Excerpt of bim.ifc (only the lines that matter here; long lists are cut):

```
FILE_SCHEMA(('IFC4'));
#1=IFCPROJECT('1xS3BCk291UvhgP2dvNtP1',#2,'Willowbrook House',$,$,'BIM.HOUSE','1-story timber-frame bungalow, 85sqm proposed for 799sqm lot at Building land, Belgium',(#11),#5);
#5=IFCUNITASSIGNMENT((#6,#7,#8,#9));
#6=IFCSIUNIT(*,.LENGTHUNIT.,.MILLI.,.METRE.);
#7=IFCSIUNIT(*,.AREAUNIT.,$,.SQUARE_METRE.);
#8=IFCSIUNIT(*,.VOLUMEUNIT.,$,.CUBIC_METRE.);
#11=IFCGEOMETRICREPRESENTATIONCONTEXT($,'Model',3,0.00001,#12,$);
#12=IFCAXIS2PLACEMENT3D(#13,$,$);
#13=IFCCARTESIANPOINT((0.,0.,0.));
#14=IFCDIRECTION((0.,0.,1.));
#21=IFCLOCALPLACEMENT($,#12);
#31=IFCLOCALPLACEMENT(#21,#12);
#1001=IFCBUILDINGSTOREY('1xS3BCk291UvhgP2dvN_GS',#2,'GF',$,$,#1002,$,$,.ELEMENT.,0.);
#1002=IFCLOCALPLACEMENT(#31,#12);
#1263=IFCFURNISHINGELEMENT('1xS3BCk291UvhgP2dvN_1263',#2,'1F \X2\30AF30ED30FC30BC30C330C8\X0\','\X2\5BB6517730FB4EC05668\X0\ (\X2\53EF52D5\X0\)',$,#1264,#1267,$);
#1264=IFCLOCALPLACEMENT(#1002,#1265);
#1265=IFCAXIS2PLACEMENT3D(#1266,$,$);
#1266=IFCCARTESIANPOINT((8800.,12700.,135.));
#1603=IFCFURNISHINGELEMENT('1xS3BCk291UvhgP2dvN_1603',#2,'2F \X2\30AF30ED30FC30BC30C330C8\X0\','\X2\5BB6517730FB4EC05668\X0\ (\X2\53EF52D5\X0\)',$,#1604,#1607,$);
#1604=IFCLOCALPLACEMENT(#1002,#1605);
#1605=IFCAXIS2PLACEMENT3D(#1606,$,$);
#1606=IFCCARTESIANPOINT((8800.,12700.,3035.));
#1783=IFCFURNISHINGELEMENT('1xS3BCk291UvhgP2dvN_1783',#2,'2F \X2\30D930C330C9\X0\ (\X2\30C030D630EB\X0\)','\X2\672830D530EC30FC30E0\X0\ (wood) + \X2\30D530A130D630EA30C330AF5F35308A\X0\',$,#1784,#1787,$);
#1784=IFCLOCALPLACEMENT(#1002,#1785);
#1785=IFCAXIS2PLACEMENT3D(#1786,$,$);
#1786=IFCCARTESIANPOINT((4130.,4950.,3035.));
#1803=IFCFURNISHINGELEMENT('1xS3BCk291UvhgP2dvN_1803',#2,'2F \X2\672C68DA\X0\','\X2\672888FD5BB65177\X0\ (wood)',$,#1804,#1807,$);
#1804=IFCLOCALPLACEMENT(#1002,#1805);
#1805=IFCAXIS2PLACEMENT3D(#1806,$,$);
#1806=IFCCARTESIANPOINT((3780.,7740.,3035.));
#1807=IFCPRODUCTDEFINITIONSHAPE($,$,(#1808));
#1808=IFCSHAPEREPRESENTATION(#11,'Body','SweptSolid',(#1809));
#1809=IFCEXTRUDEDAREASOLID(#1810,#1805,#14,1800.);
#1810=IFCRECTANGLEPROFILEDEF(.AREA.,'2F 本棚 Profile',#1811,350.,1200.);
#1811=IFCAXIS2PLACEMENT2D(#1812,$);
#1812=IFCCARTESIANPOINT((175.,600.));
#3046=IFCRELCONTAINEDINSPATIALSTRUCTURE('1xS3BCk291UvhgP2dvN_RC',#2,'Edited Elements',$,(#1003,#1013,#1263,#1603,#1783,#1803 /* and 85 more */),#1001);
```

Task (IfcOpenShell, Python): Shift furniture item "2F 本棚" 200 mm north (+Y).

```python
import ifcopenshell
import ifcopenshell.api.geometry
import ifcopenshell.util.placement
import ifcopenshell.util.unit

model = ifcopenshell.open("bim.ifc")
unit_scale = ifcopenshell.util.unit.calculate_unit_scale(model)

item = model.by_id(1803)
matrix = ifcopenshell.util.placement.get_local_placement(item.ObjectPlacement)
matrix[1, 3] += 0.2 / unit_scale
ifcopenshell.api.geometry.edit_object_placement(model, product=item, matrix=matrix, is_si=False)

print(ifcopenshell.util.placement.get_local_placement(item.ObjectPlacement).round(3) + 0.0)

model.write("bim-out.ifc")
```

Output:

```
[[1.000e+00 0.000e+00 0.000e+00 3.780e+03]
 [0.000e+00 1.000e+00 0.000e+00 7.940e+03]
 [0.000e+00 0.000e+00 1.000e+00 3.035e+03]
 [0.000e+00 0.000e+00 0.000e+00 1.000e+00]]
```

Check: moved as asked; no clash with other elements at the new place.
